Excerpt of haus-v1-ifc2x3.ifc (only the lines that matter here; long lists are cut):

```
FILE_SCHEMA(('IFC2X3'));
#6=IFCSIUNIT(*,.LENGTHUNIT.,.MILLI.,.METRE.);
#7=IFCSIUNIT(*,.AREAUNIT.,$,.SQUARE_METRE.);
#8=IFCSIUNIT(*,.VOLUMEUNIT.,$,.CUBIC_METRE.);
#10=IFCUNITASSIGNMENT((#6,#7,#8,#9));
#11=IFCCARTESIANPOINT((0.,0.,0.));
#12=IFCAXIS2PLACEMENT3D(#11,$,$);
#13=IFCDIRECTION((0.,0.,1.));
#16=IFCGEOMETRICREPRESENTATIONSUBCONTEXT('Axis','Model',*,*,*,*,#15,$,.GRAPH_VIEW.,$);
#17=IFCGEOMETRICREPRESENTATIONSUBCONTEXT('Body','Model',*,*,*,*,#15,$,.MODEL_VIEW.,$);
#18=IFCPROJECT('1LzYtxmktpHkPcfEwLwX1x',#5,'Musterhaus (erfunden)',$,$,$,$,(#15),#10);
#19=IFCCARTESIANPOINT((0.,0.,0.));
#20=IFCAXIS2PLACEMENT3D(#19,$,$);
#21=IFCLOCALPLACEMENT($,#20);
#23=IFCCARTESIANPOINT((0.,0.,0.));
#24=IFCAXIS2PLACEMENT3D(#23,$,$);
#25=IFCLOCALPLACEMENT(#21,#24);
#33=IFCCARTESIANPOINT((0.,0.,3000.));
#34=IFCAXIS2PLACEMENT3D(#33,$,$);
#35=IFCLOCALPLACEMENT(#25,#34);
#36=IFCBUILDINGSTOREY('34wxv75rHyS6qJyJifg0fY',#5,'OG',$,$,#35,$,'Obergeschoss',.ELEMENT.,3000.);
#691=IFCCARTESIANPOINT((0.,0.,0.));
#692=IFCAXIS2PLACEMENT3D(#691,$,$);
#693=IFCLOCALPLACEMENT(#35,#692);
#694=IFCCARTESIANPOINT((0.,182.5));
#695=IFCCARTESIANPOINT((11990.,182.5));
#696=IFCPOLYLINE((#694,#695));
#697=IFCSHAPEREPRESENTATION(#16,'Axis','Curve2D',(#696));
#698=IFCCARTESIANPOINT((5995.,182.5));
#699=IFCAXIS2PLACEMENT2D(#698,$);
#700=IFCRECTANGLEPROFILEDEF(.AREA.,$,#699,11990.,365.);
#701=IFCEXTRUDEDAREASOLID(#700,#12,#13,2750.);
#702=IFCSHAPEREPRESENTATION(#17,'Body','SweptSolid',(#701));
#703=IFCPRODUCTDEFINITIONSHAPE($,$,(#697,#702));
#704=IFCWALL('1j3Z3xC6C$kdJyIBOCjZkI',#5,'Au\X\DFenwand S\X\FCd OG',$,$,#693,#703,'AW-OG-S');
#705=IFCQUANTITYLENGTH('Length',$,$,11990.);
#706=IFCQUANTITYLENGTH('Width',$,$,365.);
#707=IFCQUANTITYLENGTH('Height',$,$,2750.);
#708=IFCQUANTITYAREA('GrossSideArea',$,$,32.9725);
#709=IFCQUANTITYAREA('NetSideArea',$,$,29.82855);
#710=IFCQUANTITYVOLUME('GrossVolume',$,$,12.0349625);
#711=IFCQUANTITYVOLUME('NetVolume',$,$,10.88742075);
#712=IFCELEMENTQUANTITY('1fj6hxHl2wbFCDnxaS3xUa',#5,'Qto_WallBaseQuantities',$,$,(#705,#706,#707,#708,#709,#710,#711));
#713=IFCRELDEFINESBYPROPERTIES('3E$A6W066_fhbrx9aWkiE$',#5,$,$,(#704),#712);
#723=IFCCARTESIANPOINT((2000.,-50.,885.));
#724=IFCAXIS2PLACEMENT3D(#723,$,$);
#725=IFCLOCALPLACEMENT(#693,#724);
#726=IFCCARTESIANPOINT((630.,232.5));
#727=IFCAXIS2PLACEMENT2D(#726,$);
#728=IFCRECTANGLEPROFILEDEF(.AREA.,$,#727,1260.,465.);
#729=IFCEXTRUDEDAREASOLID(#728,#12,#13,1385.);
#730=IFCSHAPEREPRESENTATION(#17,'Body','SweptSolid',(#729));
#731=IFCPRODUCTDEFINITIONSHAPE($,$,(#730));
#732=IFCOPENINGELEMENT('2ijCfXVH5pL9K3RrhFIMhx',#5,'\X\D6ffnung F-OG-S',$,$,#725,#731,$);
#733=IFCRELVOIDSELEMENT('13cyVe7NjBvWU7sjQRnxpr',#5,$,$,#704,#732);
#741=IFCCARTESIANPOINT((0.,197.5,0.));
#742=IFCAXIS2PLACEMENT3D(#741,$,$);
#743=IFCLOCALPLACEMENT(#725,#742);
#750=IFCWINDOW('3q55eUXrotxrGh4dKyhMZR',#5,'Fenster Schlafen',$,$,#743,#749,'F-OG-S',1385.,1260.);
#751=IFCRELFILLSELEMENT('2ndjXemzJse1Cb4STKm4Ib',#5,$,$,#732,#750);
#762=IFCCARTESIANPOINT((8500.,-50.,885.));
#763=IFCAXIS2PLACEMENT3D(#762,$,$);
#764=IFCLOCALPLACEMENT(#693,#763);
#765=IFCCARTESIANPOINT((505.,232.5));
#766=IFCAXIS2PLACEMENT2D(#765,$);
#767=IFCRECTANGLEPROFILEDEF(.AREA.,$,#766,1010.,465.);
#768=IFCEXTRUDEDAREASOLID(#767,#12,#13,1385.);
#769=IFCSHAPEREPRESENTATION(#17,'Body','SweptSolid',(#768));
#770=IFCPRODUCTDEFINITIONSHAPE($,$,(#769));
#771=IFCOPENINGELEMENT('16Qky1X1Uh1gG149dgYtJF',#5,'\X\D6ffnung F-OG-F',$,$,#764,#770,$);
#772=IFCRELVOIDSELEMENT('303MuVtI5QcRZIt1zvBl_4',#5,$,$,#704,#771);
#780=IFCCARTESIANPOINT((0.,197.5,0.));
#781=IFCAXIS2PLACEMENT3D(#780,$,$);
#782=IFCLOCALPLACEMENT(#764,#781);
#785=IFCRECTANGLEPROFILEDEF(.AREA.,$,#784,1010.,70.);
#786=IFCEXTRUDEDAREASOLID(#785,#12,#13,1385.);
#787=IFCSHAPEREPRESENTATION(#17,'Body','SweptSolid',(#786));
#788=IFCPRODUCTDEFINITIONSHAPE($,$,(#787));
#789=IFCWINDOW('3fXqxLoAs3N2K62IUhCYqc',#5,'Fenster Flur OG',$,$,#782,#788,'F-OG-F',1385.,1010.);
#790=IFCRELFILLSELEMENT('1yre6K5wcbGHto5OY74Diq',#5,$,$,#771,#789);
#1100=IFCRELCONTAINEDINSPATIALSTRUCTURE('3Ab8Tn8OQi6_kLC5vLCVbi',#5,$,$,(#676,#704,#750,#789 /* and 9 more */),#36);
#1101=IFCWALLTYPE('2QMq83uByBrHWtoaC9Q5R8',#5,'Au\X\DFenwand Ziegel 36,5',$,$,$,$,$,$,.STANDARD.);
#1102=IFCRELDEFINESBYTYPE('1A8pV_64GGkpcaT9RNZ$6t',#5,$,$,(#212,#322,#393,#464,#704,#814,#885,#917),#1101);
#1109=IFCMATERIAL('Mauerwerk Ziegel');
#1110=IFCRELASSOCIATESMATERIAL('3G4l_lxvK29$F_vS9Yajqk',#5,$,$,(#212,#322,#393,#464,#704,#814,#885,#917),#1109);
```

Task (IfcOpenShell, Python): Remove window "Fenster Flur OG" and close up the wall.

```python
import ifcopenshell
import ifcopenshell.api.feature
import ifcopenshell.api.pset
import ifcopenshell.api.root
import ifcopenshell.geom
import ifcopenshell.util.element
import ifcopenshell.util.shape
import ifcopenshell.util.unit

model = ifcopenshell.open("haus-v1-ifc2x3.ifc")
area_scale = ifcopenshell.util.unit.calculate_unit_scale(model, "AREAUNIT")
volume_scale = ifcopenshell.util.unit.calculate_unit_scale(model, "VOLUMEUNIT")
settings = ifcopenshell.geom.settings()


def volume(element):
    """Net volume in cubic metres, openings subtracted."""
    shape = ifcopenshell.geom.create_shape(settings, element)
    return ifcopenshell.util.shape.get_volume(shape.geometry)


window = model.by_id(789)
opening = window.FillsVoids[0].RelatingOpeningElement
wall = opening.VoidsElements[0].RelatingBuildingElement
before = volume(wall)

ifcopenshell.api.root.remove_product(model, product=window)
ifcopenshell.api.feature.remove_feature(model, feature=opening)

after = volume(wall)
thickness = 0.365  # wall thickness in metres

# Update the wall's stored quantities.
qto = model.by_id(ifcopenshell.util.element.get_pset(wall, "Qto_WallBaseQuantities", should_inherit=False)["id"])
ifcopenshell.api.pset.edit_qto(model, qto=qto, properties={
    "NetSideArea": after / thickness / area_scale,
    "NetVolume": after / volume_scale,
})

print(f"wall volume {before:.3f} -> {after:.3f} m3")

model.write("haus-v1-ifc2x3_rev.ifc")
```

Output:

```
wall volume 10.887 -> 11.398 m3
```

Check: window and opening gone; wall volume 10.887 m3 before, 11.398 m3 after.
